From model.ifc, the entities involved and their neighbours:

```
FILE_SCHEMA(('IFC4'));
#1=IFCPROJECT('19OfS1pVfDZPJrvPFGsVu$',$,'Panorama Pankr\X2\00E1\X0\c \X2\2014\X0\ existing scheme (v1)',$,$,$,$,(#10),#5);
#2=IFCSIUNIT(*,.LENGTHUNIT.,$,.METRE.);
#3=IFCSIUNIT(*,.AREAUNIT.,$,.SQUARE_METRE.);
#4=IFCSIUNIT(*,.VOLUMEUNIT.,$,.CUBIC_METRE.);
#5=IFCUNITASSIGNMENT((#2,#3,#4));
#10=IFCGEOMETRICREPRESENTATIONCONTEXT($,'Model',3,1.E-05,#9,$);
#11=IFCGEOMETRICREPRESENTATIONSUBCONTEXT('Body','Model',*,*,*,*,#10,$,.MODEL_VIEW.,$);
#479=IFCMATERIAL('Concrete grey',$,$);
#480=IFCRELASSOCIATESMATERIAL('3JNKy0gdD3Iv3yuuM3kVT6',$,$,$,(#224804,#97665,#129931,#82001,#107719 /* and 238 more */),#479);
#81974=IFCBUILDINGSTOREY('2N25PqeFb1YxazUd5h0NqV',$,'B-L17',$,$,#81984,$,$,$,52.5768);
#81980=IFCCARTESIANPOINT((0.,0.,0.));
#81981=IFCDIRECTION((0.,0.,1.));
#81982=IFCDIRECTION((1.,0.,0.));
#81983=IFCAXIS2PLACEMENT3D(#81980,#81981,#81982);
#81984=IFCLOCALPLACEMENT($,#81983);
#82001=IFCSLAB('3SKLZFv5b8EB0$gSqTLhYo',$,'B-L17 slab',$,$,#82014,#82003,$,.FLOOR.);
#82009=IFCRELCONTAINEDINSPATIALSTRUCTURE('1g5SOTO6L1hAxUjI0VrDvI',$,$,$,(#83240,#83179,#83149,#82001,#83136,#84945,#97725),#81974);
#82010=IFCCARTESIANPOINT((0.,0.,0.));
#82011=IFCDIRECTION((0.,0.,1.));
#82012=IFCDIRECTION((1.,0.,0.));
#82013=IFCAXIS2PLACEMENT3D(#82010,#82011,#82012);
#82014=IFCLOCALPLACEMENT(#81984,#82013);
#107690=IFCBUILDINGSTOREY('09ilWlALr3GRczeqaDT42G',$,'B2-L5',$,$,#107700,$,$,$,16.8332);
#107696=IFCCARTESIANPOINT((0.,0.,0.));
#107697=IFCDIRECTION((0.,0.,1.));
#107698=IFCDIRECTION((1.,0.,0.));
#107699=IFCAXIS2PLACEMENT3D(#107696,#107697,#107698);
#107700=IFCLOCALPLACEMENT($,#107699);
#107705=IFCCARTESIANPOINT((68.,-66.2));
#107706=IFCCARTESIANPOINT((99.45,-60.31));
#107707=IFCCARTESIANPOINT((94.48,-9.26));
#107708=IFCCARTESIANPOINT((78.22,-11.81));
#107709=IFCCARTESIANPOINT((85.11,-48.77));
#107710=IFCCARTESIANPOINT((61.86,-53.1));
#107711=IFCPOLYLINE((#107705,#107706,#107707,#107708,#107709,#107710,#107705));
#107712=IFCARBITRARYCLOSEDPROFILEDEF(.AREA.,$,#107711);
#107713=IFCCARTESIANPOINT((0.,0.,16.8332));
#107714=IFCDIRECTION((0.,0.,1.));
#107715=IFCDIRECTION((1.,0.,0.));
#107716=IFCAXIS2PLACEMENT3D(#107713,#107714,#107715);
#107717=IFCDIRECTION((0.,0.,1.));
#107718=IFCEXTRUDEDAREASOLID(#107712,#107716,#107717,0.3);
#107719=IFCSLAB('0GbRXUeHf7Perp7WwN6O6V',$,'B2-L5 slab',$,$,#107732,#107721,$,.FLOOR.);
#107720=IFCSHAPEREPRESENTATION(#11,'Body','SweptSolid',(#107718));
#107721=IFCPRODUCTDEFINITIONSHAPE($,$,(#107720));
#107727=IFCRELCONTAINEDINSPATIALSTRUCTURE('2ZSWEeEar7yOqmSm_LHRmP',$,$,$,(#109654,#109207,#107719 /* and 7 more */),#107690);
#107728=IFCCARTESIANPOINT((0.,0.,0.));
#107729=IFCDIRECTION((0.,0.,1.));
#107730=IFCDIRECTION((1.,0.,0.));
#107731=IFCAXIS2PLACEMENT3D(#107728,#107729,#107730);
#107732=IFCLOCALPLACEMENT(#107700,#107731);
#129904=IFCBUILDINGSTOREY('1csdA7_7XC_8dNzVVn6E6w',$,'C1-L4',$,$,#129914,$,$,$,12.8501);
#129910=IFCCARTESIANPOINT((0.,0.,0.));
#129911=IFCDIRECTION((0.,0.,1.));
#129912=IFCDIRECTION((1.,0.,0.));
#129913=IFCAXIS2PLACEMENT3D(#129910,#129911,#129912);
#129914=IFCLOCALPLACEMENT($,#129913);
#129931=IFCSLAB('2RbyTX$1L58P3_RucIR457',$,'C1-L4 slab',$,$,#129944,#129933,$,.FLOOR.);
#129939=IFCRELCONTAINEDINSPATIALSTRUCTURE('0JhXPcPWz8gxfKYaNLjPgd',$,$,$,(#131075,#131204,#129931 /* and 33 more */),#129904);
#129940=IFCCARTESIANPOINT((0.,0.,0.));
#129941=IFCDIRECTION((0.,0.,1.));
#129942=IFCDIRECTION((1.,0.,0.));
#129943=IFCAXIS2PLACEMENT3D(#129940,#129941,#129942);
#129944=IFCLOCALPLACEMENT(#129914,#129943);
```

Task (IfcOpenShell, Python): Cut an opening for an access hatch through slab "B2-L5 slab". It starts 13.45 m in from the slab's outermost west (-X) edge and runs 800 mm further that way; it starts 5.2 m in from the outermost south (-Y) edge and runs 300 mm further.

```python
import numpy as np
import ifcopenshell
import ifcopenshell.api.feature
import ifcopenshell.api.geometry
import ifcopenshell.api.root
import ifcopenshell.geom
import ifcopenshell.util.placement
import ifcopenshell.util.representation
import ifcopenshell.util.shape
import ifcopenshell.util.unit

model = ifcopenshell.open("model.ifc")
unit_scale = ifcopenshell.util.unit.calculate_unit_scale(model)
settings = ifcopenshell.geom.settings()


def volume(element):
    """Net volume in cubic metres, openings subtracted."""
    shape = ifcopenshell.geom.create_shape(settings, element)
    return ifcopenshell.util.shape.get_volume(shape.geometry)


slab = model.by_id(107719)
before = volume(slab)

# Extent in the slab's own axes, in metres. The edges named are its -X and -Y sides.
slab_shape = ifcopenshell.geom.create_shape(settings, slab)
vertices = ifcopenshell.util.shape.get_vertices(slab_shape.geometry)
x_min, y_min, bottom = vertices.min(axis=0)
top = vertices[:, 2].max()

opening = ifcopenshell.api.root.create_entity(model, ifc_class="IfcOpeningElement", name="Access hatch opening", predefined_type="OPENING")
context = ifcopenshell.util.representation.get_context(model, "Model", "Body", "MODEL_VIEW")
width, depth = 0.8, 0.3
outline = [(0.0, 0.0), (width, 0.0), (width, depth), (0.0, depth), (0.0, 0.0)]
# Overshoot both faces by 50 mm so the cut is clean.
shape = ifcopenshell.api.geometry.add_slab_representation(
    model, context=context, depth=top - bottom + 0.1, polyline=outline
)
ifcopenshell.api.geometry.assign_representation(model, product=opening, representation=shape)

matrix = ifcopenshell.util.placement.get_local_placement(slab.ObjectPlacement)
matrix[:, 3] = matrix @ np.append(np.array([x_min + 13.45, y_min + 5.2, bottom - 0.05]) / unit_scale, 1.0)
ifcopenshell.api.geometry.edit_object_placement(model, product=opening, matrix=matrix, is_si=False)
ifcopenshell.api.feature.add_feature(model, feature=opening, element=slab)

after = volume(slab)

print(f"slab volume {before:.3f} -> {after:.3f} m3")

model.write("model_v2.ifc")
```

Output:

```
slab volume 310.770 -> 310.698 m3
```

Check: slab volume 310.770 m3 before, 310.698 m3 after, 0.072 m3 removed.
